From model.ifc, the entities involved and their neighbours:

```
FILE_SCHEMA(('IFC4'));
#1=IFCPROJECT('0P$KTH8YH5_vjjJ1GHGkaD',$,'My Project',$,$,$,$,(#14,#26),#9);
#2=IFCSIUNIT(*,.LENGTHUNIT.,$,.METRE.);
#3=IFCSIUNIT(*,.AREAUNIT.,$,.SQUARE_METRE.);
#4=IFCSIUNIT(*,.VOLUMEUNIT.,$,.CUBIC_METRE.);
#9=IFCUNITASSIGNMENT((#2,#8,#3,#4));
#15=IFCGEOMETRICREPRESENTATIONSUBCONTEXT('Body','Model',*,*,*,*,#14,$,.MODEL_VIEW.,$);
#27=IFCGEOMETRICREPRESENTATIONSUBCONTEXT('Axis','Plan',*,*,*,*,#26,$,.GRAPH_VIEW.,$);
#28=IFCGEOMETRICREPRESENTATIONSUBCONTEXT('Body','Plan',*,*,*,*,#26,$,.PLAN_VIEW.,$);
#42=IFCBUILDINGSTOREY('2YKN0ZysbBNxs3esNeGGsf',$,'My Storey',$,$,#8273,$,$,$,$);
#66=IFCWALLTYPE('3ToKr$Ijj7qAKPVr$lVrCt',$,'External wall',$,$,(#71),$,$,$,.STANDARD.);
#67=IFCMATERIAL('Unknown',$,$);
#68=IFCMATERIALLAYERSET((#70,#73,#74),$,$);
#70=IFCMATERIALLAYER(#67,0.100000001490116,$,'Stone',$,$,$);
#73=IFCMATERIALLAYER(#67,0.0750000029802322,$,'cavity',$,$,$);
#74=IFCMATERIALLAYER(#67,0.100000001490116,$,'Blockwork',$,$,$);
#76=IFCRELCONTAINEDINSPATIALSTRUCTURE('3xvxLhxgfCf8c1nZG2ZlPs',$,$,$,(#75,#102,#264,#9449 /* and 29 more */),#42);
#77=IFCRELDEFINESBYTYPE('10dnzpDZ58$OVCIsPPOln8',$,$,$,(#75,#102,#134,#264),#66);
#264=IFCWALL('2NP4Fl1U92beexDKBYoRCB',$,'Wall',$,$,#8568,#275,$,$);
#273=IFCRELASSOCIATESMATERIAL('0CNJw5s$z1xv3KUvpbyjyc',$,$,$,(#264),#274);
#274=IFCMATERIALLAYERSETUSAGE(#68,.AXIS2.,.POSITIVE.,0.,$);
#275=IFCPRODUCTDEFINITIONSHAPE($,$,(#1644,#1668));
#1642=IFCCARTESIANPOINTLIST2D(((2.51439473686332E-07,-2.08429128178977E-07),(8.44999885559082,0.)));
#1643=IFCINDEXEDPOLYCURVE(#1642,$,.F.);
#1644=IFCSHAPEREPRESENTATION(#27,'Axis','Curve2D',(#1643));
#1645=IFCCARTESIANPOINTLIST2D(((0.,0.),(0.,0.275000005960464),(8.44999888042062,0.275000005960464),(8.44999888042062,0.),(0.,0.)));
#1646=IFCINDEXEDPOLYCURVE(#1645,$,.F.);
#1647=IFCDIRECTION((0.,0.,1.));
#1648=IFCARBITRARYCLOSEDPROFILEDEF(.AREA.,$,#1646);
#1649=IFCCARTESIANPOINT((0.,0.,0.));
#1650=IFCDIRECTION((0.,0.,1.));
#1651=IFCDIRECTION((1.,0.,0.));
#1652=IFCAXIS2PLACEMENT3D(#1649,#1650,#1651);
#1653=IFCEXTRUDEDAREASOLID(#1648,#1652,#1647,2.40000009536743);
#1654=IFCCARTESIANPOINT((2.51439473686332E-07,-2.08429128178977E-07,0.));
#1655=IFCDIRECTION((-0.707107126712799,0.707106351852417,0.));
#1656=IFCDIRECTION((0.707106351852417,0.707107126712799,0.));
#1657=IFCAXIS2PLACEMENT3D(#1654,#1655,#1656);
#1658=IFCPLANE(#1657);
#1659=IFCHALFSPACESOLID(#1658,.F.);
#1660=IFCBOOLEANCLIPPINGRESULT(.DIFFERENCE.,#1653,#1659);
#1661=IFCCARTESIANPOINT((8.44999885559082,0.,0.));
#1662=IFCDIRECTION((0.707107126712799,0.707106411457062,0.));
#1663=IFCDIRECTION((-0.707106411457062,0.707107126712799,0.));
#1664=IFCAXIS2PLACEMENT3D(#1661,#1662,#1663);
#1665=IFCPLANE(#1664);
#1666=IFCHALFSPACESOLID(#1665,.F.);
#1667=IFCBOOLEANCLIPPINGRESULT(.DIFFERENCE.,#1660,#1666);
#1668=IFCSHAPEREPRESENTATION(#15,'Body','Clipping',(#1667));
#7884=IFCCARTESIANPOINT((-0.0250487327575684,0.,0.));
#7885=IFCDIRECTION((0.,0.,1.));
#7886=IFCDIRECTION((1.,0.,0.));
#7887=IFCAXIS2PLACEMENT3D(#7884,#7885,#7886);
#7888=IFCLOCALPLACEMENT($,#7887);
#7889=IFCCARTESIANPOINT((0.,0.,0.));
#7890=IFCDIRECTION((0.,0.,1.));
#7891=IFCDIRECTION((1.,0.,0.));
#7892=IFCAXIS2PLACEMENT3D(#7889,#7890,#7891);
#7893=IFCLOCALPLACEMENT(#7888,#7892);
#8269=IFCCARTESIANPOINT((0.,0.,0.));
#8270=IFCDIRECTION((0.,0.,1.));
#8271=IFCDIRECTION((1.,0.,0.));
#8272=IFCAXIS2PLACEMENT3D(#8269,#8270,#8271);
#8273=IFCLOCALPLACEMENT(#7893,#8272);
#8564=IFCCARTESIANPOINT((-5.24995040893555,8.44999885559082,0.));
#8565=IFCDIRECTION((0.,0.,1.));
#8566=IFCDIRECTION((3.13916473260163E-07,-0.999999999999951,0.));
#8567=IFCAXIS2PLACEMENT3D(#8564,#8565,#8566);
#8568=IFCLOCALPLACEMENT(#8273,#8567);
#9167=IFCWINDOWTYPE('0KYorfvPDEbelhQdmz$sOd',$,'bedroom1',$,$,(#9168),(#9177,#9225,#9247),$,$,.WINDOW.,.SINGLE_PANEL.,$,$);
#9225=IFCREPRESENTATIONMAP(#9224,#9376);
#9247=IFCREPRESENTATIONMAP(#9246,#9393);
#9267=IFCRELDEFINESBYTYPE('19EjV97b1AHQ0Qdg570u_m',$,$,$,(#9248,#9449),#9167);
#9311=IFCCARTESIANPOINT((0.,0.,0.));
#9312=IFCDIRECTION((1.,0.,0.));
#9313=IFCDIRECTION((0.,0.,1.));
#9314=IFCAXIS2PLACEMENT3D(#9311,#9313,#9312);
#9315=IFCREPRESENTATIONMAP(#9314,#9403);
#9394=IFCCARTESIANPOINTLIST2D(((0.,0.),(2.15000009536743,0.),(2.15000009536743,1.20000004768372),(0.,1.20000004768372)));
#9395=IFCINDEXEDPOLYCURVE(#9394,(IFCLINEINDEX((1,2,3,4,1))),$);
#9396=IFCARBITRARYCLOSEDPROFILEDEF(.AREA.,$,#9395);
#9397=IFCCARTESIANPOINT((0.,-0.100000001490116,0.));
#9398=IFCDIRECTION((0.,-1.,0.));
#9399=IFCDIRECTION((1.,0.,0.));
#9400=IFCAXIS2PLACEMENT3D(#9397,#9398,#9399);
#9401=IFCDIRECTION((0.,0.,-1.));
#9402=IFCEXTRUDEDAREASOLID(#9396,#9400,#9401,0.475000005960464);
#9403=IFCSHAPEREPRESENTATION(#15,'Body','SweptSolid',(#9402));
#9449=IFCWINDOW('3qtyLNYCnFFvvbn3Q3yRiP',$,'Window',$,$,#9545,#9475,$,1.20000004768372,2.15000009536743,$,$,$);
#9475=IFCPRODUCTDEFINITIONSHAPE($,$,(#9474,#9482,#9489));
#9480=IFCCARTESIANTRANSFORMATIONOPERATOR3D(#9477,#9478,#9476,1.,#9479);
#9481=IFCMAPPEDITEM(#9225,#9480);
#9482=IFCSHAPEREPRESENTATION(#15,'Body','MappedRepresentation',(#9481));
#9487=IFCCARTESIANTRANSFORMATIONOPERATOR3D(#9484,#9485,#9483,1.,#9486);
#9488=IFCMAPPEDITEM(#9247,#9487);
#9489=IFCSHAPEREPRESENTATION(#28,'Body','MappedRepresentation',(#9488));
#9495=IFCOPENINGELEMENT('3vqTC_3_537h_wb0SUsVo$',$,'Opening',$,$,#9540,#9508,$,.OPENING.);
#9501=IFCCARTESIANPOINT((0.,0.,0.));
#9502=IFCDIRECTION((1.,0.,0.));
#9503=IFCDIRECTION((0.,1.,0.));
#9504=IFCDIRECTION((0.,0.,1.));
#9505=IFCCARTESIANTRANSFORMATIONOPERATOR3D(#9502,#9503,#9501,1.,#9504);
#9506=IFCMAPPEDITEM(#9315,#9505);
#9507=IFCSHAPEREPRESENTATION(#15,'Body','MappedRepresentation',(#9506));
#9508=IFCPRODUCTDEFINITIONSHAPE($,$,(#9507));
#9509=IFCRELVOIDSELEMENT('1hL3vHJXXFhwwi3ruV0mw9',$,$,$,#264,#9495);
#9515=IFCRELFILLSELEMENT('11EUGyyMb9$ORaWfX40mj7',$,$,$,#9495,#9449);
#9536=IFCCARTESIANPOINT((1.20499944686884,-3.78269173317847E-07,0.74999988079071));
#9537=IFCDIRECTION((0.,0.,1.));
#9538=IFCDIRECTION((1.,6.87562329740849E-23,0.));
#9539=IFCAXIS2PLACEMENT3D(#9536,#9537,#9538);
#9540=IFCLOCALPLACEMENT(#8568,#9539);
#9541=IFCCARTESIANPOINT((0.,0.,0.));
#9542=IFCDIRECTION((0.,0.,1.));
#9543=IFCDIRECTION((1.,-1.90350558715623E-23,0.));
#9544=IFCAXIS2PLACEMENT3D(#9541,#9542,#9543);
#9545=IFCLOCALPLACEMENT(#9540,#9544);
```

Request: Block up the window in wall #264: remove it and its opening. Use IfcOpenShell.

```python
import ifcopenshell
import ifcopenshell.api.feature
import ifcopenshell.api.root
import ifcopenshell.geom
import ifcopenshell.util.shape

model = ifcopenshell.open("model.ifc")
settings = ifcopenshell.geom.settings()


def volume(element):
    """Net volume in cubic metres, openings subtracted."""
    shape = ifcopenshell.geom.create_shape(settings, element)
    return ifcopenshell.util.shape.get_volume(shape.geometry)


window = model.by_id(9449)
opening = window.FillsVoids[0].RelatingOpeningElement
wall = opening.VoidsElements[0].RelatingBuildingElement
before = volume(wall)

ifcopenshell.api.root.remove_product(model, product=window)
ifcopenshell.api.feature.remove_feature(model, feature=opening)

after = volume(wall)

print(f"wall volume {before:.3f} -> {after:.3f} m3")

model.write("model_v2.ifc")
```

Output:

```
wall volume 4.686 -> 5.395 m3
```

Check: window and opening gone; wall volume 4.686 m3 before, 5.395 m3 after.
